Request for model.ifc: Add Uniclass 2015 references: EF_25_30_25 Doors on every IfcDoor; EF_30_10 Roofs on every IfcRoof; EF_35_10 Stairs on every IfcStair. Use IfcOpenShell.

First a look at what the model holds.

```python
import ifcopenshell

model = ifcopenshell.open("model.ifc")
print(model.schema)
print("classifications:", [c.Name for c in model.by_type("IfcClassification")])
for ifc_class in ("IfcDoor", "IfcRoof", "IfcStair", "IfcWall", "IfcWindow"):
    print(ifc_class, len(model.by_type(ifc_class)))
```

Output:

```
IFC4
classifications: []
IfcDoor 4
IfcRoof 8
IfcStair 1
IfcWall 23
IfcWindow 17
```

```python
import ifcopenshell
import ifcopenshell.api.classification

model = ifcopenshell.open("model.ifc")

system = ifcopenshell.api.classification.add_classification(model, classification="Uniclass 2015")

codes = {
    "IfcDoor": ("EF_25_30_25", "Doors"),
    "IfcRoof": ("EF_30_10", "Roofs"),
    "IfcStair": ("EF_35_10", "Stairs"),
}
for ifc_class, (code, name) in codes.items():
    products = model.by_type(ifc_class)
    ifcopenshell.api.classification.add_reference(
        model, products=products, classification=system, identification=code, name=name
    )
    print(code, len(products))

model.write("model_rev.ifc")
```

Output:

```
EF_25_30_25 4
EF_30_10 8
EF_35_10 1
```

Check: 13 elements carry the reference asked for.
